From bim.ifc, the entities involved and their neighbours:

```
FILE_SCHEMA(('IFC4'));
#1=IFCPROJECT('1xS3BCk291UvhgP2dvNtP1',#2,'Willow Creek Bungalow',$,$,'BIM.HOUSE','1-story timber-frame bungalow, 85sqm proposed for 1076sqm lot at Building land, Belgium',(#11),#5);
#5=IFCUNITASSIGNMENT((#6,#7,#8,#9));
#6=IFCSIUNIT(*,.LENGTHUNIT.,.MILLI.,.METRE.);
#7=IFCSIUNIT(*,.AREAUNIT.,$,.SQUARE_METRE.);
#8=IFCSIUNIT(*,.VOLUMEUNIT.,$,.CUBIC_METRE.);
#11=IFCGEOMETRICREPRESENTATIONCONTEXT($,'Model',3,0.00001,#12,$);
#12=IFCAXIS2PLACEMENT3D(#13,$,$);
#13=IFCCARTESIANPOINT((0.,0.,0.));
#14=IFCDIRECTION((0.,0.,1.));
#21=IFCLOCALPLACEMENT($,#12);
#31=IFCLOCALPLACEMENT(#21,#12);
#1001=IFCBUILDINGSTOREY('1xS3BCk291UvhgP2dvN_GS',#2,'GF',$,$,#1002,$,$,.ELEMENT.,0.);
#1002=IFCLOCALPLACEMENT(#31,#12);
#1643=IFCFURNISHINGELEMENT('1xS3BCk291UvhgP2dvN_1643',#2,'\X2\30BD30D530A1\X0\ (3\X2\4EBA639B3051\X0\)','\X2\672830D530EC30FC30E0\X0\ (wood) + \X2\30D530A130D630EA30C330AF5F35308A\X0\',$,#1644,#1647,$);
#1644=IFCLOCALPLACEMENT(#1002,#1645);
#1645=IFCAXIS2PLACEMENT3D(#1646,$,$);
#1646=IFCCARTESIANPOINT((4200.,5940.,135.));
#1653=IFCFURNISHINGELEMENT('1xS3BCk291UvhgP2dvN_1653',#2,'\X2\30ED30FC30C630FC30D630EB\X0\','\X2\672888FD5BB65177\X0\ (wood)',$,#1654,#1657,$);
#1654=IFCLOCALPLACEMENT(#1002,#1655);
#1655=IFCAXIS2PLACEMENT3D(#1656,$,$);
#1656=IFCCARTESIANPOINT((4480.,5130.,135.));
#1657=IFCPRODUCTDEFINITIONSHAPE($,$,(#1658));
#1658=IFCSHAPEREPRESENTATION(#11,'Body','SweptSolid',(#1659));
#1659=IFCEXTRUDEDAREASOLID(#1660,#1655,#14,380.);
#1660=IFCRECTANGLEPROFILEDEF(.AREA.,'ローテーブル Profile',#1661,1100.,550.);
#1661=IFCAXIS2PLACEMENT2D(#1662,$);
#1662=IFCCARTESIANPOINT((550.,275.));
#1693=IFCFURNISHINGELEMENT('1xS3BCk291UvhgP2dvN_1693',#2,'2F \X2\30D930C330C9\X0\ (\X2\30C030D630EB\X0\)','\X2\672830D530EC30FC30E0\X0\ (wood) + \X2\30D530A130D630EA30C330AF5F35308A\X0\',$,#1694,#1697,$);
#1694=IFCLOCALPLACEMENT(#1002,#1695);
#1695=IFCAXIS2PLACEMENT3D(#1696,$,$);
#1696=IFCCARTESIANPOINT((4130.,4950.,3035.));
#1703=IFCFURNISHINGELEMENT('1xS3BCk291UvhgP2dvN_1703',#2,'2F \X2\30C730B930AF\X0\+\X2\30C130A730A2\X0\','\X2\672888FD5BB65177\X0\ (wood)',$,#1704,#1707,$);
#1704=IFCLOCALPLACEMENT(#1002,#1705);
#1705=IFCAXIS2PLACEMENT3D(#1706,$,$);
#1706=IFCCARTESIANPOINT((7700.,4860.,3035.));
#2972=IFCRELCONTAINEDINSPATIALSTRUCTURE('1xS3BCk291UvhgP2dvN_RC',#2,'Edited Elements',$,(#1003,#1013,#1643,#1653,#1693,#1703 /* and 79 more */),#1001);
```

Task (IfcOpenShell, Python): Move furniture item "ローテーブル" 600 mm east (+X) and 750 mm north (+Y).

```python
import ifcopenshell
import ifcopenshell.api.geometry
import ifcopenshell.util.placement
import ifcopenshell.util.unit

model = ifcopenshell.open("bim.ifc")
unit_scale = ifcopenshell.util.unit.calculate_unit_scale(model)

item = model.by_guid("1xS3BCk291UvhgP2dvN_1653")
matrix = ifcopenshell.util.placement.get_local_placement(item.ObjectPlacement)
matrix[0, 3] += 0.6 / unit_scale
matrix[1, 3] += 0.75 / unit_scale
ifcopenshell.api.geometry.edit_object_placement(model, product=item, matrix=matrix, is_si=False)

print(ifcopenshell.util.placement.get_local_placement(item.ObjectPlacement).round(3) + 0.0)

model.write("bim-out.ifc")
```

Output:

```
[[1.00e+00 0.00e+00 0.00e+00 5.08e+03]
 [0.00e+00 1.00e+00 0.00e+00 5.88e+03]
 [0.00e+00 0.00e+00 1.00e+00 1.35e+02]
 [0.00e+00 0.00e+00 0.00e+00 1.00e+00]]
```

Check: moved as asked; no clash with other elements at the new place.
